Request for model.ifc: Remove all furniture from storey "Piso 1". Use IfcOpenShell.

First a look at what the model holds.

```python
import ifcopenshell
import ifcopenshell.util.element

model = ifcopenshell.open("model.ifc")
print(model.schema)
storey = next(s for s in model.by_type("IfcBuildingStorey") if s.Name == "Piso 1")
furniture = [e for e in ifcopenshell.util.element.get_decomposition(storey) if e.is_a("IfcFurnishingElement")]
seen = {}
for e in furniture:
    element_type = ifcopenshell.util.element.get_type(e)
    name = element_type.Name if element_type not in (None, e) else None
    seen[name] = seen.get(name, 0) + 1
for name, count in sorted(seen.items(), key=str):
    print(count, "x", name)
```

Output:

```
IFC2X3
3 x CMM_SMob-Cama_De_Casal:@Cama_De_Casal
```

```python
import ifcopenshell
import ifcopenshell.api.root
import ifcopenshell.util.element

model = ifcopenshell.open("model.ifc")

storey = next(s for s in model.by_type("IfcBuildingStorey") if s.Name == "Piso 1")
furniture = [e for e in ifcopenshell.util.element.get_decomposition(storey) if e.is_a("IfcFurnishingElement")]

for e in furniture:
    ifcopenshell.api.root.remove_product(model, product=e)
print(len(furniture), "removed")

model.write("model_updated.ifc")
```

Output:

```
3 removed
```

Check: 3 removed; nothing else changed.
